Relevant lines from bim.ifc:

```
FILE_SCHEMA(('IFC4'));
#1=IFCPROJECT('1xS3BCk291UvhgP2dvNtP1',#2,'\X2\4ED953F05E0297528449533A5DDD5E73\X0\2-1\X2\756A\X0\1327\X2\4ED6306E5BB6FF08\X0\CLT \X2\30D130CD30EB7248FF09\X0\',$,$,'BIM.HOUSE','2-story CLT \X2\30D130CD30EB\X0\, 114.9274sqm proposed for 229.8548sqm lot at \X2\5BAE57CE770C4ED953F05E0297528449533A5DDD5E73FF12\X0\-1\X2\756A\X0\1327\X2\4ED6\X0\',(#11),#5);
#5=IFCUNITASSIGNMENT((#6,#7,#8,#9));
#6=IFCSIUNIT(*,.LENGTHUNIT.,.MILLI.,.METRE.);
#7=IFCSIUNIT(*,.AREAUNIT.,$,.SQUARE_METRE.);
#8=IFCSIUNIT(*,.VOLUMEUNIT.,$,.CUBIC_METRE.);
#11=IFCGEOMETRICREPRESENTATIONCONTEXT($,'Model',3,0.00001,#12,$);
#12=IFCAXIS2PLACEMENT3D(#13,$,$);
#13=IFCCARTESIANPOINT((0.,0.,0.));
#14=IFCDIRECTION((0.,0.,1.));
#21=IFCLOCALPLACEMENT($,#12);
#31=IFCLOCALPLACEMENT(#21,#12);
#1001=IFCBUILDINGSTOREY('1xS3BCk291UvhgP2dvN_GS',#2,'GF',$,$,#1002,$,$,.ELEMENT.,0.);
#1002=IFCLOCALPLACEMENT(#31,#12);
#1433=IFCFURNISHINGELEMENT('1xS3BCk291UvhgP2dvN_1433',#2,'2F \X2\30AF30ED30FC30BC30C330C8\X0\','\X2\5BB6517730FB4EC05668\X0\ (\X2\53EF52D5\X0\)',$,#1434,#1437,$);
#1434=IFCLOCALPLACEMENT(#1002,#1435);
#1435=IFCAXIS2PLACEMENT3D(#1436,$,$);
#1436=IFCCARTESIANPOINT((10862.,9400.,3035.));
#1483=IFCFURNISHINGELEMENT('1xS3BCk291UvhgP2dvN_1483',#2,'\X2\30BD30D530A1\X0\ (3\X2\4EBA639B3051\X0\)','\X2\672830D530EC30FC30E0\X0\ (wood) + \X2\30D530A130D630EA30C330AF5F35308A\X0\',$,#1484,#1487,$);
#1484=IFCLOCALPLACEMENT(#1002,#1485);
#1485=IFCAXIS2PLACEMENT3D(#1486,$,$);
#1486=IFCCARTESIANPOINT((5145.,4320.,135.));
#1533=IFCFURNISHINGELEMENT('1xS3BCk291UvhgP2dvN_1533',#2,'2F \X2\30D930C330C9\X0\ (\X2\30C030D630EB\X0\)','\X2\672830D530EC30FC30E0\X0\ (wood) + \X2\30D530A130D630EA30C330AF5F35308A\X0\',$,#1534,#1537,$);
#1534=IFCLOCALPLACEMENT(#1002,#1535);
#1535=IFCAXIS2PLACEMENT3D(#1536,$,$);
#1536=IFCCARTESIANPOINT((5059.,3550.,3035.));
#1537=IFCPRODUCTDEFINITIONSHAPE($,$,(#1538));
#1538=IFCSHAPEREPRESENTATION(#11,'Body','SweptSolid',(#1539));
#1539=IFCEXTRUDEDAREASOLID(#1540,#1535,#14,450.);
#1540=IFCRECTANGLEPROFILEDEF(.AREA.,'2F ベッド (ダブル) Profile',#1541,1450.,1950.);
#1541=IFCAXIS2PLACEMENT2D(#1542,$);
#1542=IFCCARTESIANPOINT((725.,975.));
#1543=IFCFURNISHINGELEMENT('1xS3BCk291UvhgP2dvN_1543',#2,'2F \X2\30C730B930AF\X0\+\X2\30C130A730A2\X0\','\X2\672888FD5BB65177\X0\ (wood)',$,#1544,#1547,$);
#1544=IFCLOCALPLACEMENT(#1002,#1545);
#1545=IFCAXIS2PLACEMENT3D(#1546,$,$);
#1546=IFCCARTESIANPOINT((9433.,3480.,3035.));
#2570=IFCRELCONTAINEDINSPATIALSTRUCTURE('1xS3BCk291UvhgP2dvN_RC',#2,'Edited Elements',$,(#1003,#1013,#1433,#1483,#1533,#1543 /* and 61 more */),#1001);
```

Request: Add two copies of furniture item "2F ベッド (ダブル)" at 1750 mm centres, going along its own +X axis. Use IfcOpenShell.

```python
import ifcopenshell
import ifcopenshell.api.geometry
import ifcopenshell.api.root
import ifcopenshell.util.element
import ifcopenshell.util.placement

model = ifcopenshell.open("bim.ifc")


def reuse_history(source, copy):
    """copy_class also copies each property set's owner history, people and application; keep the originals."""
    for rel in copy.IsDefinedBy:
        if rel.is_a("IfcRelDefinesByProperties") and (history := rel.RelatingPropertyDefinition.OwnerHistory):
            rel.RelatingPropertyDefinition.OwnerHistory = source.OwnerHistory
            ifcopenshell.util.element.remove_deep2(model, history)


source = model.by_guid("1xS3BCk291UvhgP2dvN_1533")
base = ifcopenshell.util.placement.get_local_placement(source.ObjectPlacement)
step = base[:3, 0] * 1750.0

for i in range(1, 3):
    copy = ifcopenshell.api.root.copy_class(model, product=source)
    copy.Representation = ifcopenshell.util.element.copy_deep(
        model, source.Representation, exclude=["IfcGeometricRepresentationContext", "IfcRepresentationMap"]
    )
    reuse_history(source, copy)
    matrix = base.copy()
    matrix[:3, 3] += i * step
    print("added at", matrix[:3, 3].round(3) + 0.0)
    ifcopenshell.api.geometry.edit_object_placement(model, product=copy, matrix=matrix, is_si=False)

model.write("bim_rev.ifc")
```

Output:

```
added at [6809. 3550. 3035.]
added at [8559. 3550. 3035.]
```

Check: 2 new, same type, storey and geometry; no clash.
